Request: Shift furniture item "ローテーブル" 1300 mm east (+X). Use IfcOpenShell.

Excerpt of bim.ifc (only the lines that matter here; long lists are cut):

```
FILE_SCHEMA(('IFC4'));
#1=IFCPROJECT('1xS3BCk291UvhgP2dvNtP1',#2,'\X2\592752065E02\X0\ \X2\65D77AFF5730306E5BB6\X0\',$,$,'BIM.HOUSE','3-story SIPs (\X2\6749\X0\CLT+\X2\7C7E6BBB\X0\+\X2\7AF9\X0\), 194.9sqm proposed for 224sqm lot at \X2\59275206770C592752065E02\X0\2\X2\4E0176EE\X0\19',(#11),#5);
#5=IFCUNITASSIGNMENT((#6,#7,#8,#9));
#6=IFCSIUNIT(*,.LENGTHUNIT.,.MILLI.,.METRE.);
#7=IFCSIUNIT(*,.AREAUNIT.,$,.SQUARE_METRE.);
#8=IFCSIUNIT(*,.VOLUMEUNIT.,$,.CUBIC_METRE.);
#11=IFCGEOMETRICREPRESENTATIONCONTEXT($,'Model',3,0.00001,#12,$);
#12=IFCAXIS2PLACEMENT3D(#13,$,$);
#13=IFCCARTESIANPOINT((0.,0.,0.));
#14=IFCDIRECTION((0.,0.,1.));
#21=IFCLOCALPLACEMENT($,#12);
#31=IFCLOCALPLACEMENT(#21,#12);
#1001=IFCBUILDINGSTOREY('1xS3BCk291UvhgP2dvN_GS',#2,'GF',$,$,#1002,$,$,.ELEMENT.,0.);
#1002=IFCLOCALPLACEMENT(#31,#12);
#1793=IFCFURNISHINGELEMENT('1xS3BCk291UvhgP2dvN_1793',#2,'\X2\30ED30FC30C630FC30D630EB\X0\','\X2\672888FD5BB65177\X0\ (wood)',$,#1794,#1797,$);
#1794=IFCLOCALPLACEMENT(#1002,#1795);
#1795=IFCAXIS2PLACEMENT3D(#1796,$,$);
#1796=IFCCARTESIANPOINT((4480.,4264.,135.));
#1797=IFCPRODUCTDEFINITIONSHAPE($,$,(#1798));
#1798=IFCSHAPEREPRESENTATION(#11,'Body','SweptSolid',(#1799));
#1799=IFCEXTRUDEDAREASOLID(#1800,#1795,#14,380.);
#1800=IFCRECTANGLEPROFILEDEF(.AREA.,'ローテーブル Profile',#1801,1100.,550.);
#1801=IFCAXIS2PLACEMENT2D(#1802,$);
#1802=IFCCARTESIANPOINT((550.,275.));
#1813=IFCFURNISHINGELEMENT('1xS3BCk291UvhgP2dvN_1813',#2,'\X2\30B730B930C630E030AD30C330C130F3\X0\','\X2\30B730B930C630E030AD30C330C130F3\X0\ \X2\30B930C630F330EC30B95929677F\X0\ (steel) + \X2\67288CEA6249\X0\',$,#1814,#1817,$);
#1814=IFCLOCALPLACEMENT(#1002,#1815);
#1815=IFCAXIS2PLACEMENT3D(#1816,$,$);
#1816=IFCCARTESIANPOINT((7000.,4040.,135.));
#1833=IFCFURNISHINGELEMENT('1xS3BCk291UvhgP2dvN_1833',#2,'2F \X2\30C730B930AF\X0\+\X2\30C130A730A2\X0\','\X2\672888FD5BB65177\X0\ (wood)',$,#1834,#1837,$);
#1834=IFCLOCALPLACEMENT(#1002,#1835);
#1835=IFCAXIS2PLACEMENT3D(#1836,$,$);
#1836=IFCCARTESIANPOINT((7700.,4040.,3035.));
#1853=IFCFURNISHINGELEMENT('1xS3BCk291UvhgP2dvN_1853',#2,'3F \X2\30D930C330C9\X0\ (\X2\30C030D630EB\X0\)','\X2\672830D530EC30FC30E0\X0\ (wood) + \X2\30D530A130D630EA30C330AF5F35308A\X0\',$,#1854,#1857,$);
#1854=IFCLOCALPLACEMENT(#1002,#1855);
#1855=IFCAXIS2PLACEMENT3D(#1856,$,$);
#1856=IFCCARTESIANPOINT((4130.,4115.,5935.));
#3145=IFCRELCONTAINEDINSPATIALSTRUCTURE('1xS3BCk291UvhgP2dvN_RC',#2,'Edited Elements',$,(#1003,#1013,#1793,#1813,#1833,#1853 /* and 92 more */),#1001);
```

```python
import ifcopenshell
import ifcopenshell.api.geometry
import ifcopenshell.util.placement
import ifcopenshell.util.unit

model = ifcopenshell.open("bim.ifc")
unit_scale = ifcopenshell.util.unit.calculate_unit_scale(model)

item = model.by_guid("1xS3BCk291UvhgP2dvN_1793")
matrix = ifcopenshell.util.placement.get_local_placement(item.ObjectPlacement)
matrix[0, 3] += 1.3 / unit_scale
ifcopenshell.api.geometry.edit_object_placement(model, product=item, matrix=matrix, is_si=False)

print(ifcopenshell.util.placement.get_local_placement(item.ObjectPlacement).round(3) + 0.0)

model.write("bim_updated.ifc")
```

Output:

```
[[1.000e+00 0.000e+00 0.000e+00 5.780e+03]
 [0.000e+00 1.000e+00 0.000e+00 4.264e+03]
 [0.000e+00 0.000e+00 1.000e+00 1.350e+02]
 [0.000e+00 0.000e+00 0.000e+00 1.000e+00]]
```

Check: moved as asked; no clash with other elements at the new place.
